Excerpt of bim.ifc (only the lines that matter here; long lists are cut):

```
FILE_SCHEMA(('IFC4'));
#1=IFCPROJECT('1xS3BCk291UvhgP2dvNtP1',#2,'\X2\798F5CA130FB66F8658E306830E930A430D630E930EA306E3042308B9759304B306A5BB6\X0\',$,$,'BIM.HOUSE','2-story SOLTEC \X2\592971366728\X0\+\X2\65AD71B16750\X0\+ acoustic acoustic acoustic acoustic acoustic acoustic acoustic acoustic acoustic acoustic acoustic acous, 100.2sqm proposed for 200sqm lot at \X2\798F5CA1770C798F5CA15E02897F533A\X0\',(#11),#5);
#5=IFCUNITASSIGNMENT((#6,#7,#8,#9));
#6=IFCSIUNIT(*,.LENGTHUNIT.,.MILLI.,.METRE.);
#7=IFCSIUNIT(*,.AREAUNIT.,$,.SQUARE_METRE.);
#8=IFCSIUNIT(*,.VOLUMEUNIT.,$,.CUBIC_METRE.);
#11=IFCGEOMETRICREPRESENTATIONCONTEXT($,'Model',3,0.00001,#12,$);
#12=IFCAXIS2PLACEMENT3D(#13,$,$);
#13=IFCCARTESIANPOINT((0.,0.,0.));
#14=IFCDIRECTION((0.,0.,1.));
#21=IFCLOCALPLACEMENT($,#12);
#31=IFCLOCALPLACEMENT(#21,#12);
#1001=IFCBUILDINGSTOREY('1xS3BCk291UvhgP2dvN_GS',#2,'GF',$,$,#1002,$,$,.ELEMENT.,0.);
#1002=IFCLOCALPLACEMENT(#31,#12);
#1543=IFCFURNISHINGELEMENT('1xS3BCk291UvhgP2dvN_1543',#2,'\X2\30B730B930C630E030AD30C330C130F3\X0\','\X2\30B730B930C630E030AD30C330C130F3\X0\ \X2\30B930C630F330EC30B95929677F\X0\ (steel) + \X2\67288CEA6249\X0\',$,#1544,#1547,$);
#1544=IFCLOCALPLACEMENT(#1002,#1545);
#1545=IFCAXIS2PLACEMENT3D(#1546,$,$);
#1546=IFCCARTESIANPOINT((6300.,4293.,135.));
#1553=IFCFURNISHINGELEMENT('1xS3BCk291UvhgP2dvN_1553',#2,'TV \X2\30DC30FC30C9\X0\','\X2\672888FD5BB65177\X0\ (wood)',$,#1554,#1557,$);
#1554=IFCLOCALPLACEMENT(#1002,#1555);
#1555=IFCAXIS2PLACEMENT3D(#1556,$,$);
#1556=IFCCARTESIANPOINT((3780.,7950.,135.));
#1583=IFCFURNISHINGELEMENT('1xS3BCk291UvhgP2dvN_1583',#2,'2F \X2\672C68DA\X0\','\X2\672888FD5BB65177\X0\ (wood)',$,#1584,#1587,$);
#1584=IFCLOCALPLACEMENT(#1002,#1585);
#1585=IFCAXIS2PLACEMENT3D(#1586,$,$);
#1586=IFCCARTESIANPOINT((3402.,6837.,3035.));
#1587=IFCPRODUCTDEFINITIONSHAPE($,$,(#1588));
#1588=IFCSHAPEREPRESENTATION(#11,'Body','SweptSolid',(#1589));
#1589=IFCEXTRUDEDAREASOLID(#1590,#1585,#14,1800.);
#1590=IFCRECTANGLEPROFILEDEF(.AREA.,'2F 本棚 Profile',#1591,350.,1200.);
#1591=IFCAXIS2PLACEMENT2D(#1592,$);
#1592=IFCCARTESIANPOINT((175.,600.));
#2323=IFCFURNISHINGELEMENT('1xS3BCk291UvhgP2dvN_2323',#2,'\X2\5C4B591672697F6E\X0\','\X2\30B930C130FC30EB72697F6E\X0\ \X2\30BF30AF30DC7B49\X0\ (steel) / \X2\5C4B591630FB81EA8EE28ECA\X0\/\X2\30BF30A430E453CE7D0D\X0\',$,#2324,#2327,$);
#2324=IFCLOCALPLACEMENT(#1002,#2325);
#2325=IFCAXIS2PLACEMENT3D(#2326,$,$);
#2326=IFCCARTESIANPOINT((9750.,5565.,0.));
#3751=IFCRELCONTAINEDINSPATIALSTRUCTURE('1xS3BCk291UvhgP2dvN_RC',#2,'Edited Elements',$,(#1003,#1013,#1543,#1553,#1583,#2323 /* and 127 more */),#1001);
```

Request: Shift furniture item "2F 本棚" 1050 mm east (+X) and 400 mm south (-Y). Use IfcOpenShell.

```python
import ifcopenshell
import ifcopenshell.api.geometry
import ifcopenshell.util.placement
import ifcopenshell.util.unit

model = ifcopenshell.open("bim.ifc")
unit_scale = ifcopenshell.util.unit.calculate_unit_scale(model)

item = model.by_guid("1xS3BCk291UvhgP2dvN_1583")
matrix = ifcopenshell.util.placement.get_local_placement(item.ObjectPlacement)
matrix[0, 3] += 1.05 / unit_scale
matrix[1, 3] -= 0.4 / unit_scale
ifcopenshell.api.geometry.edit_object_placement(model, product=item, matrix=matrix, is_si=False)

print(ifcopenshell.util.placement.get_local_placement(item.ObjectPlacement).round(3) + 0.0)

model.write("bim_v2.ifc")
```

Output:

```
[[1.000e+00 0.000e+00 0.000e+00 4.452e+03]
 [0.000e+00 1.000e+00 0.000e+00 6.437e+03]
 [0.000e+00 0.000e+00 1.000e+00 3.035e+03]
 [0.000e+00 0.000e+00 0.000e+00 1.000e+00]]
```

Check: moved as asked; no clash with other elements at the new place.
